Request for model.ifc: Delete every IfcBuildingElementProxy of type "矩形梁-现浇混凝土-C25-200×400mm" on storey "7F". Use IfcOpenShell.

First a look at what the model holds.

```python
import ifcopenshell
import ifcopenshell.util.element

model = ifcopenshell.open("model.ifc")
print(model.schema)
storey = next(s for s in model.by_type("IfcBuildingStorey") if s.Name == "7F")
proxies = [e for e in ifcopenshell.util.element.get_decomposition(storey) if e.is_a("IfcBuildingElementProxy")]
seen = {}
for e in proxies:
    element_type = ifcopenshell.util.element.get_type(e)
    name = element_type.Name if element_type not in (None, e) else None
    seen[name] = seen.get(name, 0) + 1
for name, count in sorted(seen.items(), key=str):
    print(count, "x", name)
```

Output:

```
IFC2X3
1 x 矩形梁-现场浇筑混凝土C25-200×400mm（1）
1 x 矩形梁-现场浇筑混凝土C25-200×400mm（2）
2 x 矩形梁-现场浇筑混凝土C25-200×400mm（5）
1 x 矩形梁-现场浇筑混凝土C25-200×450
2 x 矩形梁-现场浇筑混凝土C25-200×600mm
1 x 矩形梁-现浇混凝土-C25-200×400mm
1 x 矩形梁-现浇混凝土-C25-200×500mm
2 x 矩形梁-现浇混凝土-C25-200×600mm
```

```python
import ifcopenshell
import ifcopenshell.api.root
import ifcopenshell.util.element

model = ifcopenshell.open("model.ifc")

storey = next(s for s in model.by_type("IfcBuildingStorey") if s.Name == "7F")
proxies = [e for e in ifcopenshell.util.element.get_decomposition(storey) if e.is_a("IfcBuildingElementProxy")]
targets = [e for e in proxies if (t := ifcopenshell.util.element.get_type(e)) not in (None, e) and t.Name == "矩形梁-现浇混凝土-C25-200×400mm"]

for e in targets:
    ifcopenshell.api.root.remove_product(model, product=e)
print(len(targets), "removed")

model.write("model_v2.ifc")
```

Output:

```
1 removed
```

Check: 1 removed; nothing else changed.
